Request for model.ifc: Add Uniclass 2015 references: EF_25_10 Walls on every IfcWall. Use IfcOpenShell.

First a look at what the model holds.

```python
import ifcopenshell

model = ifcopenshell.open("model.ifc")
print(model.schema)
print("classifications:", [c.Name for c in model.by_type("IfcClassification")])
for ifc_class in ("IfcDoor", "IfcRoof", "IfcStair", "IfcWall", "IfcWindow"):
    print(ifc_class, len(model.by_type(ifc_class)))
```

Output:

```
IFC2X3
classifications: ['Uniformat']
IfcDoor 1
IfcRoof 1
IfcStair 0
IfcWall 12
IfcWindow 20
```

```python
import ifcopenshell
import ifcopenshell.api.classification

model = ifcopenshell.open("model.ifc")

# IFC2X3 requires Source and Edition and has no link from the project to the system.
system = model.create_entity("IfcClassification", Source="NBS", Edition="2015", Name="Uniclass 2015")

codes = {
    "IfcWall": ("EF_25_10", "Walls"),
}
for ifc_class, (code, name) in codes.items():
    products = model.by_type(ifc_class)
    ifcopenshell.api.classification.add_reference(
        model, products=products, classification=system, identification=code, name=name
    )
    print(code, len(products))

model.write("model_edited.ifc")
```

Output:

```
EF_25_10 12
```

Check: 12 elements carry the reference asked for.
